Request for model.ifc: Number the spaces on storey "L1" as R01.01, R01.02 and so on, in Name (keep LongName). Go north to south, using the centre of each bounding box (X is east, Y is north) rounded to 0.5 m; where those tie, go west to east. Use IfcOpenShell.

First a look at what the model holds.

```python
import ifcopenshell
import ifcopenshell.util.element
import ifcopenshell.util.placement

model = ifcopenshell.open("model.ifc")
print(model.schema)
storey = next(s for s in model.by_type("IfcBuildingStorey") if s.Name == "L1")
spaces = [e for e in ifcopenshell.util.element.get_decomposition(storey) if e.is_a("IfcSpace")]
for e in sorted(spaces, key=lambda e: e.id()):
    origin = ifcopenshell.util.placement.get_local_placement(e.ObjectPlacement)[:3, 3]
    print(e.id(), e.Name, e.LongName, origin.round(2) + 0.0, sep=" | ")
```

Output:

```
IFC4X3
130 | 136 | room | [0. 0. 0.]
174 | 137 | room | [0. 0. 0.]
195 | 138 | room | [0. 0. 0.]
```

```python
import ifcopenshell
import ifcopenshell.geom
import ifcopenshell.util.element
import ifcopenshell.util.shape

model = ifcopenshell.open("model.ifc")
settings = ifcopenshell.geom.settings()
settings.set("use-world-coords", True)


def centre(element):
    shape = ifcopenshell.geom.create_shape(settings, element)
    return ifcopenshell.util.shape.get_bbox_centroid(shape.geometry)


storey = next(s for s in model.by_type("IfcBuildingStorey") if s.Name == "L1")
spaces = [e for e in ifcopenshell.util.element.get_decomposition(storey) if e.is_a("IfcSpace")]

# Insertion points can sit at a corner or the storey origin, so sort by the geometry (in metres).
centres = {e: centre(e) for e in spaces}
spaces.sort(key=lambda e: (-round(centres[e][1] / 0.5), centres[e][0]))

for i, e in enumerate(spaces, start=1):
    number = f"R01.{i:02d}"
    e.Name = number
    print(e.id(), number)

model.write("model_updated.ifc")
```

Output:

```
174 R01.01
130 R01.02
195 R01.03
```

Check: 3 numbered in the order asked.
